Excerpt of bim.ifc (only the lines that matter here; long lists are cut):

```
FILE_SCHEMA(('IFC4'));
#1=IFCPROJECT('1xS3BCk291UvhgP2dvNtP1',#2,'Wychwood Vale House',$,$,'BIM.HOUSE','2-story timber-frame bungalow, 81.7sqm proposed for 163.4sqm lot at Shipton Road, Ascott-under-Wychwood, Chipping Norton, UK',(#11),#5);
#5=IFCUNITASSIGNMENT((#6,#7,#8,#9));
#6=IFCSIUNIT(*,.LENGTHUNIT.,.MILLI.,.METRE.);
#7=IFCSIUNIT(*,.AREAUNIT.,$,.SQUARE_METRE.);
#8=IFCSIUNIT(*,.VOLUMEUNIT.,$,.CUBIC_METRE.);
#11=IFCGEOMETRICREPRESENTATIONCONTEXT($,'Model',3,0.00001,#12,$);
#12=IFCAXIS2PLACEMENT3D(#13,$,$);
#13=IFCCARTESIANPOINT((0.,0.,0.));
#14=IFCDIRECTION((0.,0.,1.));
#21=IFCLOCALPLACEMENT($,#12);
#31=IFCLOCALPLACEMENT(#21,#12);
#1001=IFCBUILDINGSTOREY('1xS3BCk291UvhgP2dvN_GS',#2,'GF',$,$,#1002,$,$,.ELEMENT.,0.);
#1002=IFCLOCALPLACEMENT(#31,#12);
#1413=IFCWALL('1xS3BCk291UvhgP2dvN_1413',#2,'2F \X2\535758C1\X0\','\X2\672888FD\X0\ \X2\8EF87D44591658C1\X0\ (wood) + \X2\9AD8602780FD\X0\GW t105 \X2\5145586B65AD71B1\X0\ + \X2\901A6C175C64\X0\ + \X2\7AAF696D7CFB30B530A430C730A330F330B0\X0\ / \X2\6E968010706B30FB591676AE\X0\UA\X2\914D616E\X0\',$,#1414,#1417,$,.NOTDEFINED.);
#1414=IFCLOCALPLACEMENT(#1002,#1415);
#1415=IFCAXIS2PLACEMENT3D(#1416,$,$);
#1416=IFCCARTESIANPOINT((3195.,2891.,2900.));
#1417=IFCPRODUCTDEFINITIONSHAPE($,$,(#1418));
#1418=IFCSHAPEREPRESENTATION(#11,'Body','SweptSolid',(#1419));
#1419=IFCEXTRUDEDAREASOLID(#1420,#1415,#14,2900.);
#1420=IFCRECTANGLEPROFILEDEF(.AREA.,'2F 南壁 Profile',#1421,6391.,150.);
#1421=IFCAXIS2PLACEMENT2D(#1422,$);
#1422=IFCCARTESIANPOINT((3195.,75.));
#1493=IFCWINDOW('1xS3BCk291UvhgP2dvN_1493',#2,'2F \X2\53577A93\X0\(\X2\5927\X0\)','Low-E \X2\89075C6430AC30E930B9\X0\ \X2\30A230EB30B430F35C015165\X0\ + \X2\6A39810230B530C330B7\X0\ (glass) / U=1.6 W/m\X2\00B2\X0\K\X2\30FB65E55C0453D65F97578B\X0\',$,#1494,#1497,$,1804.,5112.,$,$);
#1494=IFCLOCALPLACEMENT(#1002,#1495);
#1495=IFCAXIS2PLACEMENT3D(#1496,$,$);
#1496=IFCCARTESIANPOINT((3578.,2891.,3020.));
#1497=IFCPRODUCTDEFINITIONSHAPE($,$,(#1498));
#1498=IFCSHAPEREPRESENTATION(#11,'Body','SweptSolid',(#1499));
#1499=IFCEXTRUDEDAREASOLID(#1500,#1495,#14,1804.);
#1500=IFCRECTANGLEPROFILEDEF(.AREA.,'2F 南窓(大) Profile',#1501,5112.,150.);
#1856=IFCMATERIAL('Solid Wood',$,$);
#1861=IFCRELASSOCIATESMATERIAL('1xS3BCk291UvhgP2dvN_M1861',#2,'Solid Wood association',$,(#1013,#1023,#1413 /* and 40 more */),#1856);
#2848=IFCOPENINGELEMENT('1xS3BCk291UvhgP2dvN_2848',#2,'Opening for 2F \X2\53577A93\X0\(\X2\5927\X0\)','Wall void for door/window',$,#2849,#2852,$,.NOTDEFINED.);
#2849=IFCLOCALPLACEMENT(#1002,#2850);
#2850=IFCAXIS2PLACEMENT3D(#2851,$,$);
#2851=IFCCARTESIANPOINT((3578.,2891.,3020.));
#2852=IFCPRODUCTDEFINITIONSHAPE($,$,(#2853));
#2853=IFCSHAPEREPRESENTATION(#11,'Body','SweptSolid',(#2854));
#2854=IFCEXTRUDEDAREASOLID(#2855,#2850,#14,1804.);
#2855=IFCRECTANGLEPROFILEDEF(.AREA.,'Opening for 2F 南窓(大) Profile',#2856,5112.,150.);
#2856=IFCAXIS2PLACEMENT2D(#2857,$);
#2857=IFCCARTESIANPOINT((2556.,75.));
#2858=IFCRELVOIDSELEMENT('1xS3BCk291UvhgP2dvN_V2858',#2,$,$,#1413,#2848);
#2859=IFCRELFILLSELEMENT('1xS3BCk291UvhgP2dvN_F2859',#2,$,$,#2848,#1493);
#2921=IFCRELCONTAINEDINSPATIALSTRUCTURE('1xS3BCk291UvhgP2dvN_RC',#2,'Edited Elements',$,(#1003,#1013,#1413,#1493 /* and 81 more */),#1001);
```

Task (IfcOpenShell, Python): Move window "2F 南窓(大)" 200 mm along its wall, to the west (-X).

```python
import ifcopenshell
import ifcopenshell.api.geometry
import ifcopenshell.util.placement
import ifcopenshell.util.unit

model = ifcopenshell.open("bim.ifc")
unit_scale = ifcopenshell.util.unit.calculate_unit_scale(model)

window = model.by_guid("1xS3BCk291UvhgP2dvN_1493")
opening = window.FillsVoids[0].RelatingOpeningElement
wall = opening.VoidsElements[0].RelatingBuildingElement

wall_matrix = ifcopenshell.util.placement.get_local_placement(wall.ObjectPlacement)
shift = wall_matrix[:3, 0] * -0.2 / unit_scale
before = ifcopenshell.util.placement.get_local_placement(window.ObjectPlacement)[:3, 3].copy()

# The window is not placed relative to its opening, so move both.
for product in (opening, window):
    matrix = ifcopenshell.util.placement.get_local_placement(product.ObjectPlacement)
    matrix[:3, 3] += shift
    ifcopenshell.api.geometry.edit_object_placement(model, product=product, matrix=matrix, is_si=False)

after = ifcopenshell.util.placement.get_local_placement(window.ObjectPlacement)[:3, 3]
print("window moved by", (after - before).round(3) + 0.0)

model.write("bim_rev.ifc")
```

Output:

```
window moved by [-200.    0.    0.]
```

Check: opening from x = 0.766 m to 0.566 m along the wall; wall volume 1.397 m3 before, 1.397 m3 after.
